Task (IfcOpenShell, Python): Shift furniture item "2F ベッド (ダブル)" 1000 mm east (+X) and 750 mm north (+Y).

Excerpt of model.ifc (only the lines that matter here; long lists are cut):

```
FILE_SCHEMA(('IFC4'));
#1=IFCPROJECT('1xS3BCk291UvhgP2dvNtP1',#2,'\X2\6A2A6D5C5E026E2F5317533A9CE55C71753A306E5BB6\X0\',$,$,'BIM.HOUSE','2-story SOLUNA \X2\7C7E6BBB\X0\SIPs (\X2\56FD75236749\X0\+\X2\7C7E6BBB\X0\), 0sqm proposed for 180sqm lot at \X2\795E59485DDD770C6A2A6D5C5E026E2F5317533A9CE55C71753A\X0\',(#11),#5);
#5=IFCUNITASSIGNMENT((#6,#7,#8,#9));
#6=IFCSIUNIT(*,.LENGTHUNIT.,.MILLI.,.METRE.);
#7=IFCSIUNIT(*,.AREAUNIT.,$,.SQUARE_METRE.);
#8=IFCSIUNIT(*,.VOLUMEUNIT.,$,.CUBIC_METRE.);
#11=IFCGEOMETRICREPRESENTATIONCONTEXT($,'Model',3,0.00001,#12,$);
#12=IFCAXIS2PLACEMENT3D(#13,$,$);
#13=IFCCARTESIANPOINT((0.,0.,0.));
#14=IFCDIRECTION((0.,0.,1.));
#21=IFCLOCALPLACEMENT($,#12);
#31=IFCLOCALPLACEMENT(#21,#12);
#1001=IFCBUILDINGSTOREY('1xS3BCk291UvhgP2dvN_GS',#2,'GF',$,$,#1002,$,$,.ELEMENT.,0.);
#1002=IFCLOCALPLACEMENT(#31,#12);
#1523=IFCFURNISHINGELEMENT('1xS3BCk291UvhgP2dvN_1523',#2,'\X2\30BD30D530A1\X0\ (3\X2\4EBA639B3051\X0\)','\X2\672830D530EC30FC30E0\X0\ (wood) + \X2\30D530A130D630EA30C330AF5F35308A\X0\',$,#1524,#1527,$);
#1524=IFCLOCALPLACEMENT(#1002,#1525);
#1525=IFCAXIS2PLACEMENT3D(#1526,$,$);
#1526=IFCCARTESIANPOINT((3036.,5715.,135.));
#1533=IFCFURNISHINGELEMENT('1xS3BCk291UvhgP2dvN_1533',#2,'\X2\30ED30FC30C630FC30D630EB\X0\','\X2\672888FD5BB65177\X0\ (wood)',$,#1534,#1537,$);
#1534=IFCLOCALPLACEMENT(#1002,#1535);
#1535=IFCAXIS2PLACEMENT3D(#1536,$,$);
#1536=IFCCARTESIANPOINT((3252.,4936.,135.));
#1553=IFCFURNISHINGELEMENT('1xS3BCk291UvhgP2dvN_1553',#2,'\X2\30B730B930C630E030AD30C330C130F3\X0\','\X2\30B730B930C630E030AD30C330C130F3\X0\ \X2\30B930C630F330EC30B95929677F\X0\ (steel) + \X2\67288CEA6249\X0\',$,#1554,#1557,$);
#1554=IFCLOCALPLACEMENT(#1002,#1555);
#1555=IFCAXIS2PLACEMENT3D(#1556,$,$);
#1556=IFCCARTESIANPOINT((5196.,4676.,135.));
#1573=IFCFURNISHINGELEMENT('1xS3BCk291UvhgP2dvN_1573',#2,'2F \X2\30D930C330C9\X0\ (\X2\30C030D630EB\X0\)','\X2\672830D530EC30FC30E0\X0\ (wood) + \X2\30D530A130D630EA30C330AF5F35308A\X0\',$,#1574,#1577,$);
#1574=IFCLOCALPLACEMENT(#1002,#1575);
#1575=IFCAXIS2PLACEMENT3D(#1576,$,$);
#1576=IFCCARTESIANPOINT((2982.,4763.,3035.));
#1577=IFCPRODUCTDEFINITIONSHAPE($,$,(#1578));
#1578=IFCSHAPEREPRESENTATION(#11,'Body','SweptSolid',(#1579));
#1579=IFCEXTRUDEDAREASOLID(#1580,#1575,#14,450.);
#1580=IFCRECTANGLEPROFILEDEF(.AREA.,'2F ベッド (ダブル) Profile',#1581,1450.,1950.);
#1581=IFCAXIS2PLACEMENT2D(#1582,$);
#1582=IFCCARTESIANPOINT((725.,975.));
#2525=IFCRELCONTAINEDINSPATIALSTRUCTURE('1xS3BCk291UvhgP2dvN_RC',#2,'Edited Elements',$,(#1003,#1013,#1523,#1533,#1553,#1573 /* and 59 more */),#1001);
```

```python
import ifcopenshell
import ifcopenshell.api.geometry
import ifcopenshell.util.placement
import ifcopenshell.util.unit

model = ifcopenshell.open("model.ifc")
unit_scale = ifcopenshell.util.unit.calculate_unit_scale(model)

item = model.by_id(1573)
matrix = ifcopenshell.util.placement.get_local_placement(item.ObjectPlacement)
matrix[0, 3] += 1 / unit_scale
matrix[1, 3] += 0.75 / unit_scale
ifcopenshell.api.geometry.edit_object_placement(model, product=item, matrix=matrix, is_si=False)

print(ifcopenshell.util.placement.get_local_placement(item.ObjectPlacement).round(3) + 0.0)

model.write("model_rev.ifc")
```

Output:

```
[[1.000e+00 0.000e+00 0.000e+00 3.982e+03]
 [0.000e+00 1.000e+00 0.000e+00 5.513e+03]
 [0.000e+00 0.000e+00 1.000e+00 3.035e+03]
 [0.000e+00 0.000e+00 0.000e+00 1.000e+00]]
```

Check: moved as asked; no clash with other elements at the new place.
